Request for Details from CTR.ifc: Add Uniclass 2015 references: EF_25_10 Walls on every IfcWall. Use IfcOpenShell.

First a look at what the model holds.

```python
import ifcopenshell

model = ifcopenshell.open("Details from CTR.ifc")
print(model.schema)
print("classifications:", [c.Name for c in model.by_type("IfcClassification")])
for ifc_class in ("IfcDoor", "IfcRoof", "IfcStair", "IfcWall", "IfcWindow"):
    print(ifc_class, len(model.by_type(ifc_class)))
```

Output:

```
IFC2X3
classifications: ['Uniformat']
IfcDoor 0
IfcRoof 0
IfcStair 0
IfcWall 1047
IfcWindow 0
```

```python
import ifcopenshell
import ifcopenshell.api.classification

model = ifcopenshell.open("Details from CTR.ifc")

# IFC2X3 requires Source and Edition and has no link from the project to the system.
system = model.create_entity("IfcClassification", Source="NBS", Edition="2015", Name="Uniclass 2015")

codes = {
    "IfcWall": ("EF_25_10", "Walls"),
}
for ifc_class, (code, name) in codes.items():
    products = model.by_type(ifc_class)
    ifcopenshell.api.classification.add_reference(
        model, products=products, classification=system, identification=code, name=name
    )
    print(code, len(products))

model.write("Details from CTR-out.ifc")
```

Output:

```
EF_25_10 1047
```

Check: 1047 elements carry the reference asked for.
